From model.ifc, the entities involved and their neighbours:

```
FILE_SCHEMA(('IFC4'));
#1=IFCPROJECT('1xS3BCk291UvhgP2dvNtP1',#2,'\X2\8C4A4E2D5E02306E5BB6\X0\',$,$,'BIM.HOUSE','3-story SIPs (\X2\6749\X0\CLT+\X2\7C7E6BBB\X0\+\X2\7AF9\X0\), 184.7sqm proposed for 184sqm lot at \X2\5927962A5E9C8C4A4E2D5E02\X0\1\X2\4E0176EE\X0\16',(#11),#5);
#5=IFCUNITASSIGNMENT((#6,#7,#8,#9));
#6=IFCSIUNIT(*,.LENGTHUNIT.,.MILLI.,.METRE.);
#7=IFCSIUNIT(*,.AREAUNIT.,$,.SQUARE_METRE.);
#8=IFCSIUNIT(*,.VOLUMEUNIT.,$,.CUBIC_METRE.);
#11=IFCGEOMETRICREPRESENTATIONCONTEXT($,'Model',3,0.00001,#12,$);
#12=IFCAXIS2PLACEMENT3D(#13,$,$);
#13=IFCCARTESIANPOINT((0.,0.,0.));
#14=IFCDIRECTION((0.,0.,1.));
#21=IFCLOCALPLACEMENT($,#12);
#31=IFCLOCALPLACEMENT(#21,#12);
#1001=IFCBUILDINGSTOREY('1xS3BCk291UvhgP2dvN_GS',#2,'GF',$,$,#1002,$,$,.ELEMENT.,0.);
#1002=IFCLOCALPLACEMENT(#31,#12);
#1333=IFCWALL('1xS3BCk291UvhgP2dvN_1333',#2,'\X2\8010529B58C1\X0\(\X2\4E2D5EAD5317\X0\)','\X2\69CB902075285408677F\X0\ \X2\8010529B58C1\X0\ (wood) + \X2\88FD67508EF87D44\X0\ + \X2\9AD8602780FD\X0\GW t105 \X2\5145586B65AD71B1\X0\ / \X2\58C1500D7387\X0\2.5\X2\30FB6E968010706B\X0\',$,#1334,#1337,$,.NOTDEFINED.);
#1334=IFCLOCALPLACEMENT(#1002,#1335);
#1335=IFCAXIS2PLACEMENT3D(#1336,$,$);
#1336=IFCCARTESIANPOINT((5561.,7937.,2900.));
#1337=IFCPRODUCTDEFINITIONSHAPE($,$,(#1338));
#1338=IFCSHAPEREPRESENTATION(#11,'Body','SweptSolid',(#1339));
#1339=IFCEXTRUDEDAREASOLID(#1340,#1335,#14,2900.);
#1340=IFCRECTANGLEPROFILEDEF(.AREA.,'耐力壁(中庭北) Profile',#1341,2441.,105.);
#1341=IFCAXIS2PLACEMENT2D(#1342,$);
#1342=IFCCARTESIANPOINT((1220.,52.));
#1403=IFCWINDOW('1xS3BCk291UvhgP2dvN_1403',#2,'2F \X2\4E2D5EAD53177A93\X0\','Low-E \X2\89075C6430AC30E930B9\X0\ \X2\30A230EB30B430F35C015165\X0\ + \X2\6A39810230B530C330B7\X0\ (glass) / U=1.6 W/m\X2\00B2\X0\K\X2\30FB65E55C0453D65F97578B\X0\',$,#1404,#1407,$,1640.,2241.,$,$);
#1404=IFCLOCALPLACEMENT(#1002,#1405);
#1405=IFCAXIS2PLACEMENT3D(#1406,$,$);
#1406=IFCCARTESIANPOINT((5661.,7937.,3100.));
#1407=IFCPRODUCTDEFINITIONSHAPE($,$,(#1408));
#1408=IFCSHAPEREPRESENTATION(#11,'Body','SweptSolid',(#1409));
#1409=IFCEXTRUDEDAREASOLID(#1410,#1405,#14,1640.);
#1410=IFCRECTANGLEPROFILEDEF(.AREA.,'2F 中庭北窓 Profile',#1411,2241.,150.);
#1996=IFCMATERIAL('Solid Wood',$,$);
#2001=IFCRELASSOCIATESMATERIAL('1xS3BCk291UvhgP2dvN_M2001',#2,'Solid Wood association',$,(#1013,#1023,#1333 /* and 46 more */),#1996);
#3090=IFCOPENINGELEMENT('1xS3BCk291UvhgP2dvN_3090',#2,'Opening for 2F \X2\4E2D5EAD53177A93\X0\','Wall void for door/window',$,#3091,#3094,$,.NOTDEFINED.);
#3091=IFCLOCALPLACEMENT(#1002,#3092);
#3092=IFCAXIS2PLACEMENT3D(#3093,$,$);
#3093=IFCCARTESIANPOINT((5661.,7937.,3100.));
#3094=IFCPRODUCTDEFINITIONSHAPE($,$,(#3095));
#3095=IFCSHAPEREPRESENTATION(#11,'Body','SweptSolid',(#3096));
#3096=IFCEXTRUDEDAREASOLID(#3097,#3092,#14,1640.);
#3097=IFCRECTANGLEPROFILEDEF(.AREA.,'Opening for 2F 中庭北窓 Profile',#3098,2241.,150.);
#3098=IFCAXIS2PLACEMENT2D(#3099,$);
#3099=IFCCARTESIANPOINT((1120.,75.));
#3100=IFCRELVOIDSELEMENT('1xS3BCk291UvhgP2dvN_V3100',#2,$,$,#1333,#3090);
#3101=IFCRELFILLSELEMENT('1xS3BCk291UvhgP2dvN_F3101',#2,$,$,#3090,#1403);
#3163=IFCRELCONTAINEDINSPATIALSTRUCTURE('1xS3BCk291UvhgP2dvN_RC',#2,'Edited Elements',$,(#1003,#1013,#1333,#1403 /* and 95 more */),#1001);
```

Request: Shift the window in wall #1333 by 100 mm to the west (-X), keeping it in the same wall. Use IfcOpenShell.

```python
import ifcopenshell
import ifcopenshell.api.geometry
import ifcopenshell.util.placement

model = ifcopenshell.open("model.ifc")

window = model.by_guid("1xS3BCk291UvhgP2dvN_1403")
opening = window.FillsVoids[0].RelatingOpeningElement
wall = opening.VoidsElements[0].RelatingBuildingElement

wall_matrix = ifcopenshell.util.placement.get_local_placement(wall.ObjectPlacement)
shift = wall_matrix[:3, 0] * -100.0
before = ifcopenshell.util.placement.get_local_placement(window.ObjectPlacement)[:3, 3].copy()

# The window is not placed relative to its opening, so move both.
for product in (opening, window):
    matrix = ifcopenshell.util.placement.get_local_placement(product.ObjectPlacement)
    matrix[:3, 3] += shift
    ifcopenshell.api.geometry.edit_object_placement(model, product=product, matrix=matrix, is_si=False)

after = ifcopenshell.util.placement.get_local_placement(window.ObjectPlacement)[:3, 3]
print("window moved by", (after - before).round(3) + 0.0)

model.write("model_v2.ifc")
```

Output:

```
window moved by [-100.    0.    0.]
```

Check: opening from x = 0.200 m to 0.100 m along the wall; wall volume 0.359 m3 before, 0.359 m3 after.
